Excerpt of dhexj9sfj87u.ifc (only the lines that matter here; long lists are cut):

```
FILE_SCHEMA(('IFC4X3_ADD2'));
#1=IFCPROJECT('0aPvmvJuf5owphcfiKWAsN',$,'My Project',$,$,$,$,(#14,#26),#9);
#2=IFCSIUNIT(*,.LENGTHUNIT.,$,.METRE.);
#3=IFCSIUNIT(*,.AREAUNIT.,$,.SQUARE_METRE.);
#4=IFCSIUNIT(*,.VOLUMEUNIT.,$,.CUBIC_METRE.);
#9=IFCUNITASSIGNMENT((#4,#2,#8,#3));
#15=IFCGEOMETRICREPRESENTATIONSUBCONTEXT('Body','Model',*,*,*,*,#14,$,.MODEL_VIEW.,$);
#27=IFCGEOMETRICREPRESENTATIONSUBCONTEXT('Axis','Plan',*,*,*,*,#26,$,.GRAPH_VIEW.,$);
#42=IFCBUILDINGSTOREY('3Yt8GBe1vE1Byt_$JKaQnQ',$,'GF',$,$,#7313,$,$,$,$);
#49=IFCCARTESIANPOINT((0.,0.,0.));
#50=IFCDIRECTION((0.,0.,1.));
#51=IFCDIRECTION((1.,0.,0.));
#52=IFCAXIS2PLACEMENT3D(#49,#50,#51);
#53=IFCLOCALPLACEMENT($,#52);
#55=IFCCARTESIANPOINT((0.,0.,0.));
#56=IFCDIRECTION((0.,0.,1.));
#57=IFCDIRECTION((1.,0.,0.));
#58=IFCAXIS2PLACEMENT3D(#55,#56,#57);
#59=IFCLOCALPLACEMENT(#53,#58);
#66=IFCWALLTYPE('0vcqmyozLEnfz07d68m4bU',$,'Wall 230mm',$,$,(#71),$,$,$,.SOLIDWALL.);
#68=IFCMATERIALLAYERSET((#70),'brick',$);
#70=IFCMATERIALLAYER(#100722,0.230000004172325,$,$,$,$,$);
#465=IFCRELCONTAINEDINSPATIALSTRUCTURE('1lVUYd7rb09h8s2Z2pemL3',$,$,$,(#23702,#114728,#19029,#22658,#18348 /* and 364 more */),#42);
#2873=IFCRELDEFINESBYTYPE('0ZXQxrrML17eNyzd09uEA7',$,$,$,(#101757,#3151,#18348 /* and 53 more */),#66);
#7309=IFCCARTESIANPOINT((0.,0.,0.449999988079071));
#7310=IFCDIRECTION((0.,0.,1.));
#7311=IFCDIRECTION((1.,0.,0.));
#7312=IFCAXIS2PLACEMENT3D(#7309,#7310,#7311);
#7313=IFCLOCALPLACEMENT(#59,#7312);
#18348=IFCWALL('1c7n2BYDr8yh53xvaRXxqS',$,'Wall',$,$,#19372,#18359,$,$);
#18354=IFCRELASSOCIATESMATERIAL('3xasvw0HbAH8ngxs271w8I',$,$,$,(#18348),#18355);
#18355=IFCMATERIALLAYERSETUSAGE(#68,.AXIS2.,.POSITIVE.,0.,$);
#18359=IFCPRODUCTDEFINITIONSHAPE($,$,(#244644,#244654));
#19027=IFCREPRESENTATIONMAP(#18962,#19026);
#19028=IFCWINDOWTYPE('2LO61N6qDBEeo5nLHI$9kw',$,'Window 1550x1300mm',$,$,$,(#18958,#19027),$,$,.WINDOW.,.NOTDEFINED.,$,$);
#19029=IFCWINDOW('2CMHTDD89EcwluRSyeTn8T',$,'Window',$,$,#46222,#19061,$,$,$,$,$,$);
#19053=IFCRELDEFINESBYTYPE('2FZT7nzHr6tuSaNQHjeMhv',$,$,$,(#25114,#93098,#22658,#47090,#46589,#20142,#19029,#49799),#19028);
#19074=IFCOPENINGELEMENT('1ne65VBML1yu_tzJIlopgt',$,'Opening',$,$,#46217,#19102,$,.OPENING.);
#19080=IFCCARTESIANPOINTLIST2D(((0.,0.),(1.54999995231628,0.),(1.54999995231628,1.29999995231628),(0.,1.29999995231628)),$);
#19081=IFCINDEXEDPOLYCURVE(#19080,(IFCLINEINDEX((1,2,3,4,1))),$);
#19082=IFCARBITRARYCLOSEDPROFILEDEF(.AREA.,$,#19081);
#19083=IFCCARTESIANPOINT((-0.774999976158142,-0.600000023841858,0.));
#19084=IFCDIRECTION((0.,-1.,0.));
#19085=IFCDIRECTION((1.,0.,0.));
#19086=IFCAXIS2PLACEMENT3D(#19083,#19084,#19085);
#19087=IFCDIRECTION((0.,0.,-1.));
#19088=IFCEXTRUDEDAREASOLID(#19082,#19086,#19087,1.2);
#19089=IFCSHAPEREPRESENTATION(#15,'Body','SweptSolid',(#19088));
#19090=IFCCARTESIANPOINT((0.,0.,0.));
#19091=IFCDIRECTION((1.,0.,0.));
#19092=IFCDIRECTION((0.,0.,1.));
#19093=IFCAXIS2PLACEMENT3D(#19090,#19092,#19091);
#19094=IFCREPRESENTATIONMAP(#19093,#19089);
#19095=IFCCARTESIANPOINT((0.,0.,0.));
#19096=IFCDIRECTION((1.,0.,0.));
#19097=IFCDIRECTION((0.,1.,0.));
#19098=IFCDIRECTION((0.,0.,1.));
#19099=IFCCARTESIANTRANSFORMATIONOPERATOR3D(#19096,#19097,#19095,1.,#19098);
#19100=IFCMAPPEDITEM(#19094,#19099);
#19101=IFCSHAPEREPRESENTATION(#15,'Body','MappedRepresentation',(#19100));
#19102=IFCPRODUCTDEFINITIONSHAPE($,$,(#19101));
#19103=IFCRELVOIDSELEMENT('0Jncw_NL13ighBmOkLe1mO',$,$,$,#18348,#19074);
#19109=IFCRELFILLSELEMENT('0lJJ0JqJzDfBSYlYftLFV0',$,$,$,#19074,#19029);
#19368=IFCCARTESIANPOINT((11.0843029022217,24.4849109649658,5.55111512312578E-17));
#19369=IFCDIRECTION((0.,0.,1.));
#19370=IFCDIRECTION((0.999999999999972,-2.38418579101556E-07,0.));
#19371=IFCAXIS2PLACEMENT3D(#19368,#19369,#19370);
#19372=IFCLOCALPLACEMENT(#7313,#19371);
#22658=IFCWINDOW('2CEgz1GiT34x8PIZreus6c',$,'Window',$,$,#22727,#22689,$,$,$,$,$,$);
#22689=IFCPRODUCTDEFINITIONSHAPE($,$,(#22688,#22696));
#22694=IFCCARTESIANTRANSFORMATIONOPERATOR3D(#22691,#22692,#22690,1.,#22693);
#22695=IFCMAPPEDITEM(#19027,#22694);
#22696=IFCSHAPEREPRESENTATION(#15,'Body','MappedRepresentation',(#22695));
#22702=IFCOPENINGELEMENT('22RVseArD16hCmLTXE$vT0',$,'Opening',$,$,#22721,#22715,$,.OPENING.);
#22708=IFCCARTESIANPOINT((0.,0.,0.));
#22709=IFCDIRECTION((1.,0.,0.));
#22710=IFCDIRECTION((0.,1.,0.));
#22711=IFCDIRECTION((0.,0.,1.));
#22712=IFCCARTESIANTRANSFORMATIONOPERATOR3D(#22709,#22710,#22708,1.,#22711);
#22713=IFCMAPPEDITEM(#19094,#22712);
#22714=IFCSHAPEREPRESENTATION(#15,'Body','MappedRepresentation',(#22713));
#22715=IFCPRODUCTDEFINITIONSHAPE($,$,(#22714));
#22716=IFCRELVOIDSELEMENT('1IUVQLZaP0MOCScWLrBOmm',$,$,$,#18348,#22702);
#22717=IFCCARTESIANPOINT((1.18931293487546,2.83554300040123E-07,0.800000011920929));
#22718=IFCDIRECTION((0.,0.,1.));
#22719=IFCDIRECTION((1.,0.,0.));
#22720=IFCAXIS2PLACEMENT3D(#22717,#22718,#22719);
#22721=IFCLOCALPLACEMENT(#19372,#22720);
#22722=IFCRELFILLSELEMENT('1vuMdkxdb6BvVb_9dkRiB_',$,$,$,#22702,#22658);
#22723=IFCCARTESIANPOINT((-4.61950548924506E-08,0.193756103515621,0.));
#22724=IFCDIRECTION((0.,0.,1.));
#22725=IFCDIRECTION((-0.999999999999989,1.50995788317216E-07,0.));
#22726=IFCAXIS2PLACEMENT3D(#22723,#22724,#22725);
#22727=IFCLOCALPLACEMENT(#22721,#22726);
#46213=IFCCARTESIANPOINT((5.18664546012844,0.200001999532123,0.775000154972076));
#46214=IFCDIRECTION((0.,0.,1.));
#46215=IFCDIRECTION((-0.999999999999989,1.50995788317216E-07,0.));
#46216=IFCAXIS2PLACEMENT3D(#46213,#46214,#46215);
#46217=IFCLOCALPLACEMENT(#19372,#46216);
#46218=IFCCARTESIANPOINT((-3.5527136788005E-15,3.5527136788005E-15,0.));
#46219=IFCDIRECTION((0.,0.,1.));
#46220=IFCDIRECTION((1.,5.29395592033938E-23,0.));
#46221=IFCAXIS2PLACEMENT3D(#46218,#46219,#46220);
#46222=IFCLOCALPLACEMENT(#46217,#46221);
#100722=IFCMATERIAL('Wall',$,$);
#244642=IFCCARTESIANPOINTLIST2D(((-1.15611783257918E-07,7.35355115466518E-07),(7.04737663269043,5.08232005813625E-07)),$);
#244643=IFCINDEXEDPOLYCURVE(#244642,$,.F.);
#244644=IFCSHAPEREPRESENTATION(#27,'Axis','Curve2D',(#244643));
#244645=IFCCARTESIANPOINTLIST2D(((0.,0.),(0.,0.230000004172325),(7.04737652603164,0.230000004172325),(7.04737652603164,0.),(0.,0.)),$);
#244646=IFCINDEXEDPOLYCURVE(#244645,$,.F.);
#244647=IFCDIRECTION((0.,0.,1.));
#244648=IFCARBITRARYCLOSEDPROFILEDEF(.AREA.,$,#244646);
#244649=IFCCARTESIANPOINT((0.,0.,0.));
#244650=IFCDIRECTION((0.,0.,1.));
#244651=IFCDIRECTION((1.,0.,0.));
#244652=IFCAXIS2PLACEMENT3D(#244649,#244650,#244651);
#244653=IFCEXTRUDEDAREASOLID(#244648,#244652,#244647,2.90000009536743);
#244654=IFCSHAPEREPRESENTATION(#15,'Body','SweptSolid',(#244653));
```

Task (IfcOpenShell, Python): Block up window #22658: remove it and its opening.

```python
import ifcopenshell
import ifcopenshell.api.feature
import ifcopenshell.api.root
import ifcopenshell.geom
import ifcopenshell.util.shape

model = ifcopenshell.open("dhexj9sfj87u.ifc")
settings = ifcopenshell.geom.settings()


def volume(element):
    """Net volume in cubic metres, openings subtracted."""
    shape = ifcopenshell.geom.create_shape(settings, element)
    return ifcopenshell.util.shape.get_volume(shape.geometry)


window = model.by_guid("2CEgz1GiT34x8PIZreus6c")
opening = window.FillsVoids[0].RelatingOpeningElement
wall = opening.VoidsElements[0].RelatingBuildingElement
before = volume(wall)

ifcopenshell.api.root.remove_product(model, product=window)
ifcopenshell.api.feature.remove_feature(model, feature=opening)

after = volume(wall)

print(f"wall volume {before:.3f} -> {after:.3f} m3")

model.write("dhexj9sfj87u_updated.ifc")
```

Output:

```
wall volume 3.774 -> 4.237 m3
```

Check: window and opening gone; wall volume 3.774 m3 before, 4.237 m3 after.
